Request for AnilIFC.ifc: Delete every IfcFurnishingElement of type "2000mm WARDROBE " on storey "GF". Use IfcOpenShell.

First a look at what the model holds.

```python
import ifcopenshell
import ifcopenshell.util.element

model = ifcopenshell.open("AnilIFC.ifc")
print(model.schema)
storey = next(s for s in model.by_type("IfcBuildingStorey") if s.Name == "GF")
furniture = [e for e in ifcopenshell.util.element.get_decomposition(storey) if e.is_a("IfcFurnishingElement")]
seen = {}
for e in furniture:
    element_type = ifcopenshell.util.element.get_type(e)
    name = element_type.Name if element_type not in (None, e) else None
    seen[name] = seen.get(name, 0) + 1
for name, count in sorted(seen.items(), key=str):
    print(count, "x", name)
```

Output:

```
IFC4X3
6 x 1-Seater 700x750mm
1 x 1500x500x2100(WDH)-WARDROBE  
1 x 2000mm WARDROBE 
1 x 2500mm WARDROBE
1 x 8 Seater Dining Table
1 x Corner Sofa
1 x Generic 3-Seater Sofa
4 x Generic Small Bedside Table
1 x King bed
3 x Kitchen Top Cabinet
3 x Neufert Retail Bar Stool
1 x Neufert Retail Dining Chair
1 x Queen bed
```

```python
import ifcopenshell
import ifcopenshell.api.root
import ifcopenshell.util.element

model = ifcopenshell.open("AnilIFC.ifc")

storey = next(s for s in model.by_type("IfcBuildingStorey") if s.Name == "GF")
furniture = [e for e in ifcopenshell.util.element.get_decomposition(storey) if e.is_a("IfcFurnishingElement")]
targets = [e for e in furniture if (t := ifcopenshell.util.element.get_type(e)) not in (None, e) and t.Name == "2000mm WARDROBE "]

for e in targets:
    ifcopenshell.api.root.remove_product(model, product=e)
print(len(targets), "removed")

model.write("AnilIFC_updated.ifc")
```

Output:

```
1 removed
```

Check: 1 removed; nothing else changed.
